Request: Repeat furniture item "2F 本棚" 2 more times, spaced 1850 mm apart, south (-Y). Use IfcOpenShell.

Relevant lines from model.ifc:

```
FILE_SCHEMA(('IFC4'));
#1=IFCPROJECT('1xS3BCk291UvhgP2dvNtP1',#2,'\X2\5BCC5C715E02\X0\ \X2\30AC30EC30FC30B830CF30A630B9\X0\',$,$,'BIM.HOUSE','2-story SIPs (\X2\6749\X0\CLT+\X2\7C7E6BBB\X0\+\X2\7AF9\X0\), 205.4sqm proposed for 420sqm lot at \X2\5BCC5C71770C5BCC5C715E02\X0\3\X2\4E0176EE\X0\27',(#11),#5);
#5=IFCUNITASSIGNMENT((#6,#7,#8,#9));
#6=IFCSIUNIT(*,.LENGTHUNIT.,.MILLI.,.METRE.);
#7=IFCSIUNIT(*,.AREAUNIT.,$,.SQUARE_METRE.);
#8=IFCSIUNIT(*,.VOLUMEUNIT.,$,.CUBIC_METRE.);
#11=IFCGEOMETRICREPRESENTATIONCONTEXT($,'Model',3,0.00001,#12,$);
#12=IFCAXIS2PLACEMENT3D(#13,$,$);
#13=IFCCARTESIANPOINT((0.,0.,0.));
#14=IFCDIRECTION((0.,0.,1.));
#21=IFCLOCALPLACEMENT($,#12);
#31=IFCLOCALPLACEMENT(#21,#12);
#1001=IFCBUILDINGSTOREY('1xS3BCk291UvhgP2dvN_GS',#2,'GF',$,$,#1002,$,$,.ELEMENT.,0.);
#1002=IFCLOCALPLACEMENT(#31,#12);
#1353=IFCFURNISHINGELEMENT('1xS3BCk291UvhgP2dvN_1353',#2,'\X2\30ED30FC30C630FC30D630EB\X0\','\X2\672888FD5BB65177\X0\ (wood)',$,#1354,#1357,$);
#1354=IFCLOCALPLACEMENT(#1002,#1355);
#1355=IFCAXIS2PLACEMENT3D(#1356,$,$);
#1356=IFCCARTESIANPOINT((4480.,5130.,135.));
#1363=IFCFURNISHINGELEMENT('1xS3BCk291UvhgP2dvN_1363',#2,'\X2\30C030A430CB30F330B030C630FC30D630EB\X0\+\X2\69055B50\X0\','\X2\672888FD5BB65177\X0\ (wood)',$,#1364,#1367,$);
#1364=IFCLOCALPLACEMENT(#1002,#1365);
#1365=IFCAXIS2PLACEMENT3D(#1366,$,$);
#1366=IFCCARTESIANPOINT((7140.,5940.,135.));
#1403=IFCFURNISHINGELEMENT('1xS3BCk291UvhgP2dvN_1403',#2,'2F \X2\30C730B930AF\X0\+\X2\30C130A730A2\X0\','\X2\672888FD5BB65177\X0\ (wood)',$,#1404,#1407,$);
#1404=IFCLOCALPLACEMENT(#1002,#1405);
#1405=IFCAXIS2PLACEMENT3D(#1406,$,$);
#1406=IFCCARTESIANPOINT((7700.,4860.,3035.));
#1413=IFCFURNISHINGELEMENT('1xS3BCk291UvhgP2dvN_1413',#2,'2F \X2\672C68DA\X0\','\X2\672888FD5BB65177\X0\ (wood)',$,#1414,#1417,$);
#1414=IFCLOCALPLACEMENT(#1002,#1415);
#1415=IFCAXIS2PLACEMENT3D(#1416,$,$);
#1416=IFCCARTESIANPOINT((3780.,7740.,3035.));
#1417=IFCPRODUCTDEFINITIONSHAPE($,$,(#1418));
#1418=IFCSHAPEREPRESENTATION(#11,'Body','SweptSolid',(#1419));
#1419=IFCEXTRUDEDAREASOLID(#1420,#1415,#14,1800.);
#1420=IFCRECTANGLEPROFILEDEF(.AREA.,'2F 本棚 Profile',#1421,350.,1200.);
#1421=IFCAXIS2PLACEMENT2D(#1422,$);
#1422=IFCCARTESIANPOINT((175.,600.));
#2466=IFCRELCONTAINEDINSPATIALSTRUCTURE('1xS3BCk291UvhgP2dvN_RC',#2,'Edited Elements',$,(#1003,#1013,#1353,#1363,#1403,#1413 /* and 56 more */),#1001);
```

```python
import numpy as np
import ifcopenshell
import ifcopenshell.api.geometry
import ifcopenshell.api.root
import ifcopenshell.util.element
import ifcopenshell.util.placement
import ifcopenshell.util.unit

model = ifcopenshell.open("model.ifc")
unit_scale = ifcopenshell.util.unit.calculate_unit_scale(model)


def reuse_history(source, copy):
    """copy_class also copies each property set's owner history, people and application; keep the originals."""
    for rel in copy.IsDefinedBy:
        if rel.is_a("IfcRelDefinesByProperties") and (history := rel.RelatingPropertyDefinition.OwnerHistory):
            rel.RelatingPropertyDefinition.OwnerHistory = source.OwnerHistory
            ifcopenshell.util.element.remove_deep2(model, history)


source = model.by_guid("1xS3BCk291UvhgP2dvN_1413")
base = ifcopenshell.util.placement.get_local_placement(source.ObjectPlacement)
step = np.array([0.0, -1.0, 0.0]) * 1.85 / unit_scale

for i in range(1, 3):
    copy = ifcopenshell.api.root.copy_class(model, product=source)
    copy.Representation = ifcopenshell.util.element.copy_deep(
        model, source.Representation, exclude=["IfcGeometricRepresentationContext", "IfcRepresentationMap"]
    )
    reuse_history(source, copy)
    matrix = base.copy()
    matrix[:3, 3] += i * step
    print("added at", matrix[:3, 3].round(3) + 0.0)
    ifcopenshell.api.geometry.edit_object_placement(model, product=copy, matrix=matrix, is_si=False)

model.write("model_v2.ifc")
```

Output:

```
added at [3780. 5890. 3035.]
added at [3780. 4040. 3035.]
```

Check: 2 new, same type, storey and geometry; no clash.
